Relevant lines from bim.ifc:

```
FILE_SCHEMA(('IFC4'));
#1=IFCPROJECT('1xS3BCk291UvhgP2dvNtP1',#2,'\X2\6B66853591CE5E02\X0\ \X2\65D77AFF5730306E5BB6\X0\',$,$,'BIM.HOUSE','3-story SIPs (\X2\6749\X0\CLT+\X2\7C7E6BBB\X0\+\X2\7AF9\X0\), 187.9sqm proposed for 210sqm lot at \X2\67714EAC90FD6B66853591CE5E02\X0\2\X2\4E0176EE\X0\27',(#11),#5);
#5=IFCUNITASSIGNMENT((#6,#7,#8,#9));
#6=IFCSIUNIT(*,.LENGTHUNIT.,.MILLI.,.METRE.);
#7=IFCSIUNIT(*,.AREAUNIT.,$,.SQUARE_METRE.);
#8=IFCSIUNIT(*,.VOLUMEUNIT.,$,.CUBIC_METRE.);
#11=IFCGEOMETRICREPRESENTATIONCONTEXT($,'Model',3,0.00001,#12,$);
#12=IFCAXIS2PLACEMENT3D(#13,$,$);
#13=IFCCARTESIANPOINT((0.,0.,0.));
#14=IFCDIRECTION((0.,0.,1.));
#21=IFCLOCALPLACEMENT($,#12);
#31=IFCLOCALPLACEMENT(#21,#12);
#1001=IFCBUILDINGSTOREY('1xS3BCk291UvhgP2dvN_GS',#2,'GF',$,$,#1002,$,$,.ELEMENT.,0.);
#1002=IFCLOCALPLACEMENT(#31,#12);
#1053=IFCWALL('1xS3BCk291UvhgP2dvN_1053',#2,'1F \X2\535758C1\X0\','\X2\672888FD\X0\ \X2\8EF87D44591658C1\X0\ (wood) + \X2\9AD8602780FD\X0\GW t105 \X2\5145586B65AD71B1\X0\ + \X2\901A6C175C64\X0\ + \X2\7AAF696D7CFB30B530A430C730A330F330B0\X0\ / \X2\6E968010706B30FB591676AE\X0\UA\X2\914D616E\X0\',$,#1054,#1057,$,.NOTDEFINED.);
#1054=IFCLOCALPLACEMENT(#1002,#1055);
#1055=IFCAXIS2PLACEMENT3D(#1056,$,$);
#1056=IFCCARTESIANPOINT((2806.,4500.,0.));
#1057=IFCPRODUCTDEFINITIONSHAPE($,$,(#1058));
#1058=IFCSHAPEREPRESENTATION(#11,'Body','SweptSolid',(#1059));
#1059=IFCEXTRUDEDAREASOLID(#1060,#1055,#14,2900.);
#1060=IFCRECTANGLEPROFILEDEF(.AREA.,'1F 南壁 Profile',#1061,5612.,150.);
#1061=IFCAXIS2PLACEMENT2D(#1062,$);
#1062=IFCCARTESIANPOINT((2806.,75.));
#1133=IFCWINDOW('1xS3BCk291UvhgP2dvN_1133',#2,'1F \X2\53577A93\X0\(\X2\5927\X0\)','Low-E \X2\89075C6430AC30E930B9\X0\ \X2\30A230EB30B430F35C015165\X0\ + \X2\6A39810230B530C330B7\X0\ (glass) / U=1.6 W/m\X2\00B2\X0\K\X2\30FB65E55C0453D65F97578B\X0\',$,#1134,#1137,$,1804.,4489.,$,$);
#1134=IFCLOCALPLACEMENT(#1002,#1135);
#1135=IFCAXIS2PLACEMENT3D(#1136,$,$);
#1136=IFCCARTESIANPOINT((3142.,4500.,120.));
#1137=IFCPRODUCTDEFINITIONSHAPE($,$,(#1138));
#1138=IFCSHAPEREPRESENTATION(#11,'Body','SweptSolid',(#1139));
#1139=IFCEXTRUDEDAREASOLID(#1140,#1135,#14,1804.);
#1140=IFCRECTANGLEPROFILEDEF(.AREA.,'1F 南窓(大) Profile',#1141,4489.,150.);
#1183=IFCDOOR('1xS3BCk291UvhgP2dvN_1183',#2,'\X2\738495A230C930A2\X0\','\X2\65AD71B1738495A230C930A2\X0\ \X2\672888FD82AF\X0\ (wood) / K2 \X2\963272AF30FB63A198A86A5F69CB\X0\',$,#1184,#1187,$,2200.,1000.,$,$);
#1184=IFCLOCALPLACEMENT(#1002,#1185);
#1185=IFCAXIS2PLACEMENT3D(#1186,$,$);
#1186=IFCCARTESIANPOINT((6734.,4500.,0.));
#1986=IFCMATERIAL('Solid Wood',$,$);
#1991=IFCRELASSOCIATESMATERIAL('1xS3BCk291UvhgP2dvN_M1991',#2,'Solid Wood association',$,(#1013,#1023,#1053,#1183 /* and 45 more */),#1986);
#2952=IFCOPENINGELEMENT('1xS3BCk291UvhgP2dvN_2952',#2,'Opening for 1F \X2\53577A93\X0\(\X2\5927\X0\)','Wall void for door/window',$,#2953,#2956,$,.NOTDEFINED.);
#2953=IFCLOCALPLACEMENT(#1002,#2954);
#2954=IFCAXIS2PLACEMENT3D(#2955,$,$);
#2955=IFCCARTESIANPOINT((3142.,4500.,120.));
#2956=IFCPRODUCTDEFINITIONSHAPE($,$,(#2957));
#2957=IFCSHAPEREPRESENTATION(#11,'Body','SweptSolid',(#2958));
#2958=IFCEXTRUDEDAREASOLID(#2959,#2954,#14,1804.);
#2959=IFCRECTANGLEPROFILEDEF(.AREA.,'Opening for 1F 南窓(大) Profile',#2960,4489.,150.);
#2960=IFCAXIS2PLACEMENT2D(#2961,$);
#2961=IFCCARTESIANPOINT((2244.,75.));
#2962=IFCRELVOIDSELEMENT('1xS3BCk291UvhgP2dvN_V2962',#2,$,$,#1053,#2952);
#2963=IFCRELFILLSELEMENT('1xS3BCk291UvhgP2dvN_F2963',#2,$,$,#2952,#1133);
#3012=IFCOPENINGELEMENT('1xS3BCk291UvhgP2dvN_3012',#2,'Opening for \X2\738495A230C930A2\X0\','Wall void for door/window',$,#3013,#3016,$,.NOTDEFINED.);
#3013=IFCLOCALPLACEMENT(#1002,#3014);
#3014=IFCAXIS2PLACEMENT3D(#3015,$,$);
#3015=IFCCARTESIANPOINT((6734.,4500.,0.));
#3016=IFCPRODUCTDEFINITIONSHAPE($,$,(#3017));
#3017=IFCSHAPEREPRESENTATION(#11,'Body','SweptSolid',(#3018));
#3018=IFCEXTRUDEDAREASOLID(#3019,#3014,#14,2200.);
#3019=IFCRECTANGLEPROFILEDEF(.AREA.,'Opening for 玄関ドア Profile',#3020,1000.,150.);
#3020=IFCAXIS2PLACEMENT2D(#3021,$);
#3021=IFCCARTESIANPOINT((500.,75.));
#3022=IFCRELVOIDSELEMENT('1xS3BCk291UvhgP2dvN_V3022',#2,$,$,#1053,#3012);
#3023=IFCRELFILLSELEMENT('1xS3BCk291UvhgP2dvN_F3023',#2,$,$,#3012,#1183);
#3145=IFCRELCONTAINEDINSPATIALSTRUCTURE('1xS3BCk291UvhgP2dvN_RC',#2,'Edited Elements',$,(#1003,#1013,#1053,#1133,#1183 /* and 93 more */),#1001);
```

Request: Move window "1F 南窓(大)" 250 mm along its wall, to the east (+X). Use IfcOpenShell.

```python
import ifcopenshell
import ifcopenshell.api.geometry
import ifcopenshell.util.placement
import ifcopenshell.util.unit

model = ifcopenshell.open("bim.ifc")
unit_scale = ifcopenshell.util.unit.calculate_unit_scale(model)

window = model.by_guid("1xS3BCk291UvhgP2dvN_1133")
opening = window.FillsVoids[0].RelatingOpeningElement
wall = opening.VoidsElements[0].RelatingBuildingElement

wall_matrix = ifcopenshell.util.placement.get_local_placement(wall.ObjectPlacement)
shift = wall_matrix[:3, 0] * 0.25 / unit_scale
before = ifcopenshell.util.placement.get_local_placement(window.ObjectPlacement)[:3, 3].copy()

# The window is not placed relative to its opening, so move both.
for product in (opening, window):
    matrix = ifcopenshell.util.placement.get_local_placement(product.ObjectPlacement)
    matrix[:3, 3] += shift
    ifcopenshell.api.geometry.edit_object_placement(model, product=product, matrix=matrix, is_si=False)

after = ifcopenshell.util.placement.get_local_placement(window.ObjectPlacement)[:3, 3]
print("window moved by", (after - before).round(3) + 0.0)

model.write("bim_updated.ifc")
```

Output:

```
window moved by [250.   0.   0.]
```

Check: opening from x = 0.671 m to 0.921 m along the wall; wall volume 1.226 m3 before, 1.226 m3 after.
